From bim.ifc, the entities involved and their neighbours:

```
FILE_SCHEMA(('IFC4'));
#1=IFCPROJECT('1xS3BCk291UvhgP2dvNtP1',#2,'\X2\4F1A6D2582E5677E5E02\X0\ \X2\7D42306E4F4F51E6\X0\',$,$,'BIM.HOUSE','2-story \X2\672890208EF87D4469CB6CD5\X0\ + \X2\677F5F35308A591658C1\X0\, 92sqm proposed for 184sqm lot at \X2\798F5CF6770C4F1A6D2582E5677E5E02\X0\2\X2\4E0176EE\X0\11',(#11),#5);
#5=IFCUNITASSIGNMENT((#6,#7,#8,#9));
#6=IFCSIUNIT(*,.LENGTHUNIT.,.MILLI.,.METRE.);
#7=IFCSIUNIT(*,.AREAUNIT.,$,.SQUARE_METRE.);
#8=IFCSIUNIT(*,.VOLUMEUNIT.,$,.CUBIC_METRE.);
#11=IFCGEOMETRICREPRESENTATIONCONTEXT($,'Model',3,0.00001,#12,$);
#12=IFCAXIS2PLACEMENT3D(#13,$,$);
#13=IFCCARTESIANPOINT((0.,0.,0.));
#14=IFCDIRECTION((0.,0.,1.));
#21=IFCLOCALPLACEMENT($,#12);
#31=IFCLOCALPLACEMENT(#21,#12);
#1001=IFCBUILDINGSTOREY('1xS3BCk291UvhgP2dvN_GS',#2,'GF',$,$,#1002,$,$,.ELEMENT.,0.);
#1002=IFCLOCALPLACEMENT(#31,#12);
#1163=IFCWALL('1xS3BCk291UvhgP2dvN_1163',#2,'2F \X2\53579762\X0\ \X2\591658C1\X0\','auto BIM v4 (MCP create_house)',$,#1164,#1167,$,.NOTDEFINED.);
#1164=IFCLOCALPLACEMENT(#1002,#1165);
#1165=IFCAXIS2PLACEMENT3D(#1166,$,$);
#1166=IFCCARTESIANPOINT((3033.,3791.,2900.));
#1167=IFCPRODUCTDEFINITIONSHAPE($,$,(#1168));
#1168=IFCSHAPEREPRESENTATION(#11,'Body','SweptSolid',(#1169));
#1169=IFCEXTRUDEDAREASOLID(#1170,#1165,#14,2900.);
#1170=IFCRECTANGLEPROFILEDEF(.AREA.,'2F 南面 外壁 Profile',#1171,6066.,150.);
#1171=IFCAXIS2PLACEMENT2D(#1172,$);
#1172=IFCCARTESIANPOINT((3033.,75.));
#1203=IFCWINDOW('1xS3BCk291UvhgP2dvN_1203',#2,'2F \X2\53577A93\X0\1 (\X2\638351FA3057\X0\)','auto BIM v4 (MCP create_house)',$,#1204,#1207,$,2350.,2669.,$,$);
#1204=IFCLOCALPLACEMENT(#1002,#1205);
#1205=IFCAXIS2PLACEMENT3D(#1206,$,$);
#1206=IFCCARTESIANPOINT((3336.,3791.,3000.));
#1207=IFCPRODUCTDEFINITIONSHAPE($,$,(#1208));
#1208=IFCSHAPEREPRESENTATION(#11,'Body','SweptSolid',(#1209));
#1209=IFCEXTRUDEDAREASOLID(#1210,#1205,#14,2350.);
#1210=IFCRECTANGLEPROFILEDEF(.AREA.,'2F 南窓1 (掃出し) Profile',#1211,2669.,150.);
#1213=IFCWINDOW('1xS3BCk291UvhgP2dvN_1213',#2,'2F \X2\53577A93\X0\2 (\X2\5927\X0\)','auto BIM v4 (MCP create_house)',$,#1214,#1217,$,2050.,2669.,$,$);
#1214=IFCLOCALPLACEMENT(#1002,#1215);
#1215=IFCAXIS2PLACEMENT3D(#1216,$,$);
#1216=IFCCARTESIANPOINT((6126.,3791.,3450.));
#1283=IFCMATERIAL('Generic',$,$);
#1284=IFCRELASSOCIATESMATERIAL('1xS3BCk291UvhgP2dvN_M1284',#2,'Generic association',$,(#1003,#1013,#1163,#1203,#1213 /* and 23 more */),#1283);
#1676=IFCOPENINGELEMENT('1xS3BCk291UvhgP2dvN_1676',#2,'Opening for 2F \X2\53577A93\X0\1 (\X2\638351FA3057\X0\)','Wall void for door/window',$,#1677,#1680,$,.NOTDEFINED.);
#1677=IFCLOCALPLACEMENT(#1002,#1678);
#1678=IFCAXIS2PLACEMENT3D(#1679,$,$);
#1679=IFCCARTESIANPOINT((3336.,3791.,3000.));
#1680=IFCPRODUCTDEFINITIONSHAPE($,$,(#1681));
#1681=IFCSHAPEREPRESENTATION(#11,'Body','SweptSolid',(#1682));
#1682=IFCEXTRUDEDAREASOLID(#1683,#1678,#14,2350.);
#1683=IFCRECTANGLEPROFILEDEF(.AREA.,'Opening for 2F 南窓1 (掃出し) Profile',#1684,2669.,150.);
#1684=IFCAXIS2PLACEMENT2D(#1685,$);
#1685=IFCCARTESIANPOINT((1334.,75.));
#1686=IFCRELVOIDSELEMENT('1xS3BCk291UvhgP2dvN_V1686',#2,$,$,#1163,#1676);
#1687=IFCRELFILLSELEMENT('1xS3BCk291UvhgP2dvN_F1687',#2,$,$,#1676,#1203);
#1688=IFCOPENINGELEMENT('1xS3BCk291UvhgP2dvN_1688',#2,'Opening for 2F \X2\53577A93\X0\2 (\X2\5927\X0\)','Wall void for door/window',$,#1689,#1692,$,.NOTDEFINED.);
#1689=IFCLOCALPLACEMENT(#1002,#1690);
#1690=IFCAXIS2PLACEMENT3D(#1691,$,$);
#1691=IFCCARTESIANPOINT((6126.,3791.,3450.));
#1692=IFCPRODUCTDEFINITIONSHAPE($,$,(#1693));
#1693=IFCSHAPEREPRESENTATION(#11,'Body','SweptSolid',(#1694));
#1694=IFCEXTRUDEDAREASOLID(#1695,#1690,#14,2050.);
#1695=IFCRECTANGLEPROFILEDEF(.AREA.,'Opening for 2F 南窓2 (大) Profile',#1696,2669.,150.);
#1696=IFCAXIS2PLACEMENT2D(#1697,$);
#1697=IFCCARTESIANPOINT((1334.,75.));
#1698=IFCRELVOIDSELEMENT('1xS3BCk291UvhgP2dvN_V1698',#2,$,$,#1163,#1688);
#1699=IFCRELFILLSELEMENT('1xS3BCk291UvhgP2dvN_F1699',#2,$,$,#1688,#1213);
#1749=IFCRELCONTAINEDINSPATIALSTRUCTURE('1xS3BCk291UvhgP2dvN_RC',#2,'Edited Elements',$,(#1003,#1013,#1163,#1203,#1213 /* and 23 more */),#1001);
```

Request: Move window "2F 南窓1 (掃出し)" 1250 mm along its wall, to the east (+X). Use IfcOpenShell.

```python
import ifcopenshell
import ifcopenshell.api.geometry
import ifcopenshell.util.placement

model = ifcopenshell.open("bim.ifc")

window = model.by_guid("1xS3BCk291UvhgP2dvN_1203")
opening = window.FillsVoids[0].RelatingOpeningElement
wall = opening.VoidsElements[0].RelatingBuildingElement

wall_matrix = ifcopenshell.util.placement.get_local_placement(wall.ObjectPlacement)
shift = wall_matrix[:3, 0] * 1250.0
before = ifcopenshell.util.placement.get_local_placement(window.ObjectPlacement)[:3, 3].copy()

# The window is not placed relative to its opening, so move both.
for product in (opening, window):
    matrix = ifcopenshell.util.placement.get_local_placement(product.ObjectPlacement)
    matrix[:3, 3] += shift
    ifcopenshell.api.geometry.edit_object_placement(model, product=product, matrix=matrix, is_si=False)

after = ifcopenshell.util.placement.get_local_placement(window.ObjectPlacement)[:3, 3]
print("window moved by", (after - before).round(3) + 0.0)

model.write("bim_edited.ifc")
```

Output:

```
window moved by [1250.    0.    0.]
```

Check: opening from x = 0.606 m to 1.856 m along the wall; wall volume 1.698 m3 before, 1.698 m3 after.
